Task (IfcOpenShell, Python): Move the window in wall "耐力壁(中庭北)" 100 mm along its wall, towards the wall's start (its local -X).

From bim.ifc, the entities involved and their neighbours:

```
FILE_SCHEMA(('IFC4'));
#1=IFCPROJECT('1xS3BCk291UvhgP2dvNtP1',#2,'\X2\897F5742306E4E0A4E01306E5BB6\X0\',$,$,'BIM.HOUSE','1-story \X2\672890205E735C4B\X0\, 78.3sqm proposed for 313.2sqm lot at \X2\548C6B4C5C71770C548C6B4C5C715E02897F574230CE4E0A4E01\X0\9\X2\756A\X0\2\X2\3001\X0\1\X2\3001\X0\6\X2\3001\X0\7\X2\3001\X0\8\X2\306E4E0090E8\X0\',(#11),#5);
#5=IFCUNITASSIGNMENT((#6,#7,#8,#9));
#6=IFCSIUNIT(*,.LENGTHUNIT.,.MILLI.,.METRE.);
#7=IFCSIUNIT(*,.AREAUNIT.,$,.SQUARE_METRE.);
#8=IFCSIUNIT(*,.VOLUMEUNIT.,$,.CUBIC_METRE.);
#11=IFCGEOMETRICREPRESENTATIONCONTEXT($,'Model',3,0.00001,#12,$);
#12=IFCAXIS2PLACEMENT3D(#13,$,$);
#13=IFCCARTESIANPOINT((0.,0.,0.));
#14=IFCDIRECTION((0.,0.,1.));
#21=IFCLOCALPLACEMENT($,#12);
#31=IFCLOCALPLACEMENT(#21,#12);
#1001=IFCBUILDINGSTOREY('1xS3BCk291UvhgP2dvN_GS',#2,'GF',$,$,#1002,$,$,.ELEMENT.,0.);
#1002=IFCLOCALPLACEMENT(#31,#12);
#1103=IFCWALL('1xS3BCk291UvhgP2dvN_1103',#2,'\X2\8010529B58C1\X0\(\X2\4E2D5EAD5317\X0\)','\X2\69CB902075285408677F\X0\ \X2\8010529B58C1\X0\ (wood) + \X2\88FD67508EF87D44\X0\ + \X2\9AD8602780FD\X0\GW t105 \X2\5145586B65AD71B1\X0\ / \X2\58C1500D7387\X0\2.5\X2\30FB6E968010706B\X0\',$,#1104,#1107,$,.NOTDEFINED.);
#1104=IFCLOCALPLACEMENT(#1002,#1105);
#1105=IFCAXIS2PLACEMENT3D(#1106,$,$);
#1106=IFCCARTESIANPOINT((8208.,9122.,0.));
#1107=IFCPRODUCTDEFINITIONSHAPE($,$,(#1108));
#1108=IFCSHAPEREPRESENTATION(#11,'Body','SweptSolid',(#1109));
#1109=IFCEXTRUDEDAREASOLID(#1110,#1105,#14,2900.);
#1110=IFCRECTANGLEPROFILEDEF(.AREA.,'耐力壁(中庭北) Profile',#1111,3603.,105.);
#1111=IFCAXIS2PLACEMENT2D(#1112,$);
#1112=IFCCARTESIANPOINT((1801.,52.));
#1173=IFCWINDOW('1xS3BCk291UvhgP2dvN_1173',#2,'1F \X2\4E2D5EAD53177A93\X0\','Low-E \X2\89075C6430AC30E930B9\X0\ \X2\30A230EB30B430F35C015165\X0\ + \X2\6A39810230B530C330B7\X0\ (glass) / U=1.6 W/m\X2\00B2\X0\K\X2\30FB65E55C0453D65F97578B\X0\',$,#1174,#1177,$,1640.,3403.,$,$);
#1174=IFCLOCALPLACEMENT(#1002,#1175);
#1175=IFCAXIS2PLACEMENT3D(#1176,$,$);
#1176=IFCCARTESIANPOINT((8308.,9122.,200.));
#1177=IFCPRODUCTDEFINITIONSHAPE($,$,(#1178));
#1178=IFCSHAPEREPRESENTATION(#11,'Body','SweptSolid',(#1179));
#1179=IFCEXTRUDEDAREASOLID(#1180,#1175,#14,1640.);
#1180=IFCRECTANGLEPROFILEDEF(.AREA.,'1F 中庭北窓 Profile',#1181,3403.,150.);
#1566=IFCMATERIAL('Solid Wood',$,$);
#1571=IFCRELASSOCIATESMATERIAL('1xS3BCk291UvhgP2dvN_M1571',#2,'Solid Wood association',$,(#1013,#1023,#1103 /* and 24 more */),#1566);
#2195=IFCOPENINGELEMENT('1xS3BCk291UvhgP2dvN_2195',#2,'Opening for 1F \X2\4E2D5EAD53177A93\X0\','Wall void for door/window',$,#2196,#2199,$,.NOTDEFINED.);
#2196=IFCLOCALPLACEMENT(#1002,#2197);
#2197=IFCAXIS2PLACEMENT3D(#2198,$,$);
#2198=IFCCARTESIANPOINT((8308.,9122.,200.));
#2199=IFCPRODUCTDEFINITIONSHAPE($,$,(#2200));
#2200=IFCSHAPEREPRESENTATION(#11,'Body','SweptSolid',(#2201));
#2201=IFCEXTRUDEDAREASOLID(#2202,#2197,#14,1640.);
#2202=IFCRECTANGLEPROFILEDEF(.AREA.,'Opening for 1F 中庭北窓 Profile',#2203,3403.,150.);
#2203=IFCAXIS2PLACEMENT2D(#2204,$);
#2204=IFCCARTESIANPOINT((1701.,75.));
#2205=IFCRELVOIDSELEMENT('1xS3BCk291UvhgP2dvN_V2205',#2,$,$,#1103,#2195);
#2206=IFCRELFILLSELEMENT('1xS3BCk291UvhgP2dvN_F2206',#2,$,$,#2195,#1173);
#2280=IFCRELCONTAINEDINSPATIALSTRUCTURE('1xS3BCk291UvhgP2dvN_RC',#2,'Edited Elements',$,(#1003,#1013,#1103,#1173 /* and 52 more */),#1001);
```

```python
import ifcopenshell
import ifcopenshell.api.geometry
import ifcopenshell.util.placement

model = ifcopenshell.open("bim.ifc")

window = model.by_guid("1xS3BCk291UvhgP2dvN_1173")
opening = window.FillsVoids[0].RelatingOpeningElement
wall = opening.VoidsElements[0].RelatingBuildingElement

wall_matrix = ifcopenshell.util.placement.get_local_placement(wall.ObjectPlacement)
shift = wall_matrix[:3, 0] * -100.0
before = ifcopenshell.util.placement.get_local_placement(window.ObjectPlacement)[:3, 3].copy()

# The window is not placed relative to its opening, so move both.
for product in (opening, window):
    matrix = ifcopenshell.util.placement.get_local_placement(product.ObjectPlacement)
    matrix[:3, 3] += shift
    ifcopenshell.api.geometry.edit_object_placement(model, product=product, matrix=matrix, is_si=False)

after = ifcopenshell.util.placement.get_local_placement(window.ObjectPlacement)[:3, 3]
print("window moved by", (after - before).round(3) + 0.0)

model.write("bim_rev.ifc")
```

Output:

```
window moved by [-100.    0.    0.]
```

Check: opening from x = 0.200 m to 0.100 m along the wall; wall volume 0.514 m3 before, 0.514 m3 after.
